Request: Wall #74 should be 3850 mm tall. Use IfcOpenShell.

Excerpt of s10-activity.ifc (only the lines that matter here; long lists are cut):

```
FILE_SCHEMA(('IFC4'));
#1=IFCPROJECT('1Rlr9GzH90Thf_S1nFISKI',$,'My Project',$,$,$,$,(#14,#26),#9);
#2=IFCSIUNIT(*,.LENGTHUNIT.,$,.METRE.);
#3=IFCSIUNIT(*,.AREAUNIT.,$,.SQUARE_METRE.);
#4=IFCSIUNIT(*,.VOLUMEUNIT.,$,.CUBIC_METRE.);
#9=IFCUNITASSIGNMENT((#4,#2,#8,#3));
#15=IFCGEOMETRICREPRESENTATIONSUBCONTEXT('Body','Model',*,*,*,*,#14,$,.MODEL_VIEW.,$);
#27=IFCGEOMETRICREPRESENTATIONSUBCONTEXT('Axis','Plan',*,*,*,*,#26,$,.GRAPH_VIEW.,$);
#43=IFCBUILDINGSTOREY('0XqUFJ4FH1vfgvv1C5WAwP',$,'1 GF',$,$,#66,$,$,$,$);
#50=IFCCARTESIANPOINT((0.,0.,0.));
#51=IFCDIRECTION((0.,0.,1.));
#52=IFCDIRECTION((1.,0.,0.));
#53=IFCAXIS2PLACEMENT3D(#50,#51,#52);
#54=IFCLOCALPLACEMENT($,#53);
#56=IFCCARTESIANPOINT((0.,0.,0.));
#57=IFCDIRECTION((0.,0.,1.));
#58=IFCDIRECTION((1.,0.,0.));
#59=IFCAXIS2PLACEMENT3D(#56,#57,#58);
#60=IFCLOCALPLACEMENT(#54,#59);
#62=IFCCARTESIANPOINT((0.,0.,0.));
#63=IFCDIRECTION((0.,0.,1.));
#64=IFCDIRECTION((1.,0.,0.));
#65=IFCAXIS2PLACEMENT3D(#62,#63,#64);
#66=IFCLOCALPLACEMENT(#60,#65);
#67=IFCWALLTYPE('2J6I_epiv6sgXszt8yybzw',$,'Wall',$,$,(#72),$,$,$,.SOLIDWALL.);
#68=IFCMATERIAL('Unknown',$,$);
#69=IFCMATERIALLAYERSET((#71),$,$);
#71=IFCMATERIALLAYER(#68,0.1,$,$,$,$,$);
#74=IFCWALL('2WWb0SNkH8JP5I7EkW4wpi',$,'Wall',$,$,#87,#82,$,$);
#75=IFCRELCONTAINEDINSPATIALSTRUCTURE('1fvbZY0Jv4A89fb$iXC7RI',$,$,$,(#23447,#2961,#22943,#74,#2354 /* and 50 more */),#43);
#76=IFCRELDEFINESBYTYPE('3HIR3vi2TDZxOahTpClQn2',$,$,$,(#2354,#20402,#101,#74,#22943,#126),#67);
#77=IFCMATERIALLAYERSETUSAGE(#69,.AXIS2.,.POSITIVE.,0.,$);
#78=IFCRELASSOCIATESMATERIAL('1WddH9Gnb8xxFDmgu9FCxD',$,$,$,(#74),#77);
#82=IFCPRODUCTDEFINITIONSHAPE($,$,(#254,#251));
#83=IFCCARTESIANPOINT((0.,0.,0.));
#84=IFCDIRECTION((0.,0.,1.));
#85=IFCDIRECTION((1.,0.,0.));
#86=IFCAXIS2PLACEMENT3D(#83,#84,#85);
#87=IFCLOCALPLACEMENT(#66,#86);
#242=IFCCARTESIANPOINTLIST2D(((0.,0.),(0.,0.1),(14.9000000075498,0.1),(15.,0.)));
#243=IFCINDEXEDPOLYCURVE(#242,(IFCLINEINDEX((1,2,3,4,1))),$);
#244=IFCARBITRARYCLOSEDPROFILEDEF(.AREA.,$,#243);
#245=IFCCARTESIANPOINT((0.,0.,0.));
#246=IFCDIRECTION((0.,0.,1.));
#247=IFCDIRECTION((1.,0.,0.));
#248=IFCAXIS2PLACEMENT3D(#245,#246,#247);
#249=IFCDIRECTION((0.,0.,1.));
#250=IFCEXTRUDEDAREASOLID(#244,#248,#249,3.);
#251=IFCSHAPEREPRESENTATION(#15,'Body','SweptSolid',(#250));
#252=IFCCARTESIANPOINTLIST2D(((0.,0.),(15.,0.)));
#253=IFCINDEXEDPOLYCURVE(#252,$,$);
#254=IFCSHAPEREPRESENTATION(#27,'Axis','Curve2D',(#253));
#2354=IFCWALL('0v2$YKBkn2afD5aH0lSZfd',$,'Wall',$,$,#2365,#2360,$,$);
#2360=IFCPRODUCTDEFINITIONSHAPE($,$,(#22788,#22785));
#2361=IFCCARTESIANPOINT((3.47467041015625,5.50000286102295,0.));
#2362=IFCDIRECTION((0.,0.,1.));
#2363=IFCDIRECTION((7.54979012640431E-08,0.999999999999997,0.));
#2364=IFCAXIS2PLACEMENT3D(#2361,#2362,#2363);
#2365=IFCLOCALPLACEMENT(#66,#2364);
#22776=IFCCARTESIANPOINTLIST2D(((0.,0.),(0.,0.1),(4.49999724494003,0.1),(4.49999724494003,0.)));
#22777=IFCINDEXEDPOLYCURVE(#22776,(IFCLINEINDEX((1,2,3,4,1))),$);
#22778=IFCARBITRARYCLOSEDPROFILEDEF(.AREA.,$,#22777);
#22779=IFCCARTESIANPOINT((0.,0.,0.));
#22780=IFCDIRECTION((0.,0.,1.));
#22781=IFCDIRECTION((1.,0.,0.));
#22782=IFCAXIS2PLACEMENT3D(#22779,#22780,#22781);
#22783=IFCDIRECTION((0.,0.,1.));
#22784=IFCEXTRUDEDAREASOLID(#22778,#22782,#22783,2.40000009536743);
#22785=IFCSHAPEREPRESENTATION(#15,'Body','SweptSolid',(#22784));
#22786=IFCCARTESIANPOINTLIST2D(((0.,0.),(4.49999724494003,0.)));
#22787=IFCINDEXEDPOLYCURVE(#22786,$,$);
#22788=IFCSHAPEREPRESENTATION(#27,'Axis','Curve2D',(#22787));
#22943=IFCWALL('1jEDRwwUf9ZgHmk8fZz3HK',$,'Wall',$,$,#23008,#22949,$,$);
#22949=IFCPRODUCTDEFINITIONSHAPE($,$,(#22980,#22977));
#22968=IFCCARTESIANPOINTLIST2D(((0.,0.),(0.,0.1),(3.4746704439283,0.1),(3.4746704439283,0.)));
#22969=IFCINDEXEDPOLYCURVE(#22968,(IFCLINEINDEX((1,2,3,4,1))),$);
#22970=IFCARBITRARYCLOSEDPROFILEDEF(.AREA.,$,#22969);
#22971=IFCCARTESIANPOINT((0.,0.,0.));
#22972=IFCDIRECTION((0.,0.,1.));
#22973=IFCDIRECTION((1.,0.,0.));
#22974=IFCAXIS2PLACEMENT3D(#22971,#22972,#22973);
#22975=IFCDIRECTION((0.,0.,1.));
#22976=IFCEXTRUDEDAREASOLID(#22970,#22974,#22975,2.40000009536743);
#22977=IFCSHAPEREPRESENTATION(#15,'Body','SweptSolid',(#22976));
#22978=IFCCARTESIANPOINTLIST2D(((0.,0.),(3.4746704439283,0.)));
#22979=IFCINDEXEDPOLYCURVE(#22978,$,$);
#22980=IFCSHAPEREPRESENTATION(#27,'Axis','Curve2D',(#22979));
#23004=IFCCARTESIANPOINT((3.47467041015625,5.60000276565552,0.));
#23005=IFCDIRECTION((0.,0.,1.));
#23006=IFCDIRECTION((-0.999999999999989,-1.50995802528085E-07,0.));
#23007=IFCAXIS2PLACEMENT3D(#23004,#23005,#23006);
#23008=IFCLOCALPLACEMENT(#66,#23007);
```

```python
import ifcopenshell
import ifcopenshell.geom
import ifcopenshell.util.representation
import ifcopenshell.util.shape
import ifcopenshell.util.unit

model = ifcopenshell.open("s10-activity.ifc")
unit_scale = ifcopenshell.util.unit.calculate_unit_scale(model)
settings = ifcopenshell.geom.settings()


def volume(element):
    """Net volume in cubic metres, openings subtracted."""
    shape = ifcopenshell.geom.create_shape(settings, element)
    return ifcopenshell.util.shape.get_volume(shape.geometry)


wall = model.by_id(74)
before = volume(wall)

body = ifcopenshell.util.representation.get_representation(wall, "Model", "Body")
solid = body.Items[0]
old_height = solid.Depth
solid.Depth = 3.85 / unit_scale
after = volume(wall)

print(f"height {old_height:g} -> {solid.Depth:g}, volume {before:.3f} -> {after:.3f} m3")

model.write("s10-activity_rev.ifc")
```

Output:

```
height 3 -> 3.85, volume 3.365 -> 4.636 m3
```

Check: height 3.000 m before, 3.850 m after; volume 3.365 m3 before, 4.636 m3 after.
